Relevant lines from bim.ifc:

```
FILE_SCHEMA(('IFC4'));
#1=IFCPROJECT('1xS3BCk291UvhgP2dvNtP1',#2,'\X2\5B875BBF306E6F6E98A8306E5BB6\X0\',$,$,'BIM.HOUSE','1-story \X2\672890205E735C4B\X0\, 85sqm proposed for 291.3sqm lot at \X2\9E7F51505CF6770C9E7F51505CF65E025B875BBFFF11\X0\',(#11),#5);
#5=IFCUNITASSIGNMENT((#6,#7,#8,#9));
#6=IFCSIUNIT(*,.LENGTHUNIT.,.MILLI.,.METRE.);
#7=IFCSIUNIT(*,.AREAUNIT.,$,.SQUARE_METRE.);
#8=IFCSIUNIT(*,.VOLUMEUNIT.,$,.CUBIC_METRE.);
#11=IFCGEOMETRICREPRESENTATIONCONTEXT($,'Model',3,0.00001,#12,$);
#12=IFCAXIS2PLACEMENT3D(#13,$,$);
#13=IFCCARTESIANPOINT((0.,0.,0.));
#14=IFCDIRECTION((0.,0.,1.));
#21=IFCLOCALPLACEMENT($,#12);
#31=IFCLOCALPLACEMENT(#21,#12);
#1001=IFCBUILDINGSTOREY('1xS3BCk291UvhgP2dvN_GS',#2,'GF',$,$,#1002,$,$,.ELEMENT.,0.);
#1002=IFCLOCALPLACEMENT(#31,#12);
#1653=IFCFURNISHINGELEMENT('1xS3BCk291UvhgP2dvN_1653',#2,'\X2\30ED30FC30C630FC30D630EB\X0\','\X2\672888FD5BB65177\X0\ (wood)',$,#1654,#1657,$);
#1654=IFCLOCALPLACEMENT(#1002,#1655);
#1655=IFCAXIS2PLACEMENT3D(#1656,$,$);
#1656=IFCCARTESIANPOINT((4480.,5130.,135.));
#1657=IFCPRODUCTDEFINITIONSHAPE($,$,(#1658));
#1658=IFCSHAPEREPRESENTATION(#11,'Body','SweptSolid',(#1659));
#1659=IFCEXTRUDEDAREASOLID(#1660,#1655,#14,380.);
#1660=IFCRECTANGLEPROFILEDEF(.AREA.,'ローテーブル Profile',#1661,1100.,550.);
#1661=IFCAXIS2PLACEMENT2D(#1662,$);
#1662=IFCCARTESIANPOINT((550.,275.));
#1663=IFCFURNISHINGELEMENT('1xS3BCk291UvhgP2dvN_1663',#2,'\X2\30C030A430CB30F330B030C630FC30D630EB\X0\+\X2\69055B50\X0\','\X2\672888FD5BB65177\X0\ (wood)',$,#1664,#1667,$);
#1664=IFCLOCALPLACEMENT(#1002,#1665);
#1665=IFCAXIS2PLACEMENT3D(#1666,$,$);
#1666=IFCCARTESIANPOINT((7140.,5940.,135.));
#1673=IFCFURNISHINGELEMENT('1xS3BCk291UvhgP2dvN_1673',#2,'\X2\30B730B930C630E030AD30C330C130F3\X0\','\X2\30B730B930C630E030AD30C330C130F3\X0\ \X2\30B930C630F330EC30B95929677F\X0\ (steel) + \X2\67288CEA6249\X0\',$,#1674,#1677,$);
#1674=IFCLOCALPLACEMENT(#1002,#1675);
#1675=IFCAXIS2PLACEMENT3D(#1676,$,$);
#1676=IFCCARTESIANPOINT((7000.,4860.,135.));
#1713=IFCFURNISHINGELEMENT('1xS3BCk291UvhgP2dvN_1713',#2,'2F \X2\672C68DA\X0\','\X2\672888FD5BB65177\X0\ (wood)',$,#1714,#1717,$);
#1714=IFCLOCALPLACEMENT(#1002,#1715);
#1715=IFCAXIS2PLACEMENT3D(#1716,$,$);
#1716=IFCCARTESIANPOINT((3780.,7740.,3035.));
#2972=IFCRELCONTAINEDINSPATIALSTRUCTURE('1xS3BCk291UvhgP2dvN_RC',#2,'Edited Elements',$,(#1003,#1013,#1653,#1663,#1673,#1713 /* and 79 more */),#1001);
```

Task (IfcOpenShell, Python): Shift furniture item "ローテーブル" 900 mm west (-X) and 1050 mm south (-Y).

```python
import ifcopenshell
import ifcopenshell.api.geometry
import ifcopenshell.util.placement
import ifcopenshell.util.unit

model = ifcopenshell.open("bim.ifc")
unit_scale = ifcopenshell.util.unit.calculate_unit_scale(model)

item = model.by_id(1653)
matrix = ifcopenshell.util.placement.get_local_placement(item.ObjectPlacement)
matrix[0, 3] -= 0.9 / unit_scale
matrix[1, 3] -= 1.05 / unit_scale
ifcopenshell.api.geometry.edit_object_placement(model, product=item, matrix=matrix, is_si=False)

print(ifcopenshell.util.placement.get_local_placement(item.ObjectPlacement).round(3) + 0.0)

model.write("bim_rev.ifc")
```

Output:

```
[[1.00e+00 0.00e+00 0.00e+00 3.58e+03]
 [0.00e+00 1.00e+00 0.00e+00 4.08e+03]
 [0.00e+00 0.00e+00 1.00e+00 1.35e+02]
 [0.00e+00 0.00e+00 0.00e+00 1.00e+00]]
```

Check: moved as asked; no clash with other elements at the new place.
